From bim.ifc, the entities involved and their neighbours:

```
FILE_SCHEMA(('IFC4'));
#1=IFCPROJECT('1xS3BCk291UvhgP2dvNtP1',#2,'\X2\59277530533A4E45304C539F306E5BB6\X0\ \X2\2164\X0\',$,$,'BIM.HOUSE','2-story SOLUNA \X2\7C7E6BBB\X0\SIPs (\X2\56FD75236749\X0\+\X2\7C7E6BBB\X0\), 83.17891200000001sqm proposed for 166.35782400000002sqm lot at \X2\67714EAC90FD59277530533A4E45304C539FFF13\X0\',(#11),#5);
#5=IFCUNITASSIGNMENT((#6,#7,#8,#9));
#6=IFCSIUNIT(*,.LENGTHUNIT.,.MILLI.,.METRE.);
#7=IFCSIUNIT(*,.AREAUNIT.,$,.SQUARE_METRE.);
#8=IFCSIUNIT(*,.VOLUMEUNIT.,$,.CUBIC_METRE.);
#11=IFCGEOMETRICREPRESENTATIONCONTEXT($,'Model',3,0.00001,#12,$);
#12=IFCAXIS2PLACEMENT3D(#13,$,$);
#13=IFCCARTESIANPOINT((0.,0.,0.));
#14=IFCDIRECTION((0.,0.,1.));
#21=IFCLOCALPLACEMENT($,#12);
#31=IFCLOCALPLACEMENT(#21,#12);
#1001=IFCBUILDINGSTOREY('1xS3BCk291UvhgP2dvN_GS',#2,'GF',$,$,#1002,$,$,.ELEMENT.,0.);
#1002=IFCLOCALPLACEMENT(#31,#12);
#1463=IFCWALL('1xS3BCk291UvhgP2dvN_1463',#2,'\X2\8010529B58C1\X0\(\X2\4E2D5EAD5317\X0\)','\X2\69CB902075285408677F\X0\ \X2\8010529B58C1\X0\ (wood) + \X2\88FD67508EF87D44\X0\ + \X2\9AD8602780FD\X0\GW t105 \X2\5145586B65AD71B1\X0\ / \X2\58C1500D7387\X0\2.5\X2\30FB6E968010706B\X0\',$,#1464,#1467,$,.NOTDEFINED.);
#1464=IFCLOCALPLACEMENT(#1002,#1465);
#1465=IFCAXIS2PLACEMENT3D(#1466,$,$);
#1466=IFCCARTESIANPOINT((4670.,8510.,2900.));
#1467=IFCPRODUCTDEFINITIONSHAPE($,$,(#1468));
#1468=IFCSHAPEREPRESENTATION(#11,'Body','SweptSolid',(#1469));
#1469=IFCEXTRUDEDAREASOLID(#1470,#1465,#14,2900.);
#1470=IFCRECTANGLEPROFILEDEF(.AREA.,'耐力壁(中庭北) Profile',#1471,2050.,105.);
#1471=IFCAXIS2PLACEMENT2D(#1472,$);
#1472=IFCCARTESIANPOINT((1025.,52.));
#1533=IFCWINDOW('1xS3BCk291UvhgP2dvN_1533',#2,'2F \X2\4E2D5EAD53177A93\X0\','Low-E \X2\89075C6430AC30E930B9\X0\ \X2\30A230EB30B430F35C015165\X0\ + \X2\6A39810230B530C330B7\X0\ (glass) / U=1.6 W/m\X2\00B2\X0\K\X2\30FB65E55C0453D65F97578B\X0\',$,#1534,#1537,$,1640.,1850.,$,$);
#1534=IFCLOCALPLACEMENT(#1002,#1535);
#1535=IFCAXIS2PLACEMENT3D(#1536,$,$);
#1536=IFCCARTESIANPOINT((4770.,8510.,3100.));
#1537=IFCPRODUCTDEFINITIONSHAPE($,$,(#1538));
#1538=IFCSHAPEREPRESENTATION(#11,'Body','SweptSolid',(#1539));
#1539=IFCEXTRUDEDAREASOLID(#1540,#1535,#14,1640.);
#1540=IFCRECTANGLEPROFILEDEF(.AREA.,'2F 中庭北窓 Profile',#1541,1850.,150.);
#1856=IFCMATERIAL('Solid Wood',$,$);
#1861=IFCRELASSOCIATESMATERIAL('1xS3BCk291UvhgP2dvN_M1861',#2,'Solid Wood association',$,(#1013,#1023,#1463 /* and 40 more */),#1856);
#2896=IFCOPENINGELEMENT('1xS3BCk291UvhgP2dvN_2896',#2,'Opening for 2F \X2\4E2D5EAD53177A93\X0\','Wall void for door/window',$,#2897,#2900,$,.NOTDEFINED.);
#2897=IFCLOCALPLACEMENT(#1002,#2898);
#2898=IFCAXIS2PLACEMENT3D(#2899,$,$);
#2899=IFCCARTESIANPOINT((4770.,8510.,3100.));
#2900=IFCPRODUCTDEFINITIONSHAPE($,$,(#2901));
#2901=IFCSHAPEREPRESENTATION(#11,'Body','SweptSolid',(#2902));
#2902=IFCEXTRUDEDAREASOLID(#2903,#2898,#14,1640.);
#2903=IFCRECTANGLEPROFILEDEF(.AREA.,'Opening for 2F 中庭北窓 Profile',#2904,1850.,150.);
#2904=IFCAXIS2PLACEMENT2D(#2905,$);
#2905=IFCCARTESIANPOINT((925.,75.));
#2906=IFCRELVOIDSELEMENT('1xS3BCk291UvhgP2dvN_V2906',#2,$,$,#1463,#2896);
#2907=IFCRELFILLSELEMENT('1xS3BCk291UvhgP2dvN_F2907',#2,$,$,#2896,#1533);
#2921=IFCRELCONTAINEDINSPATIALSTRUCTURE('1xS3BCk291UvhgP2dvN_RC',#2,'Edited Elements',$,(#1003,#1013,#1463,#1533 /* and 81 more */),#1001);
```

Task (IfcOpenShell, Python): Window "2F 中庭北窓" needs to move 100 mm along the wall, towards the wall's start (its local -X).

```python
import ifcopenshell
import ifcopenshell.api.geometry
import ifcopenshell.util.placement
import ifcopenshell.util.unit

model = ifcopenshell.open("bim.ifc")
unit_scale = ifcopenshell.util.unit.calculate_unit_scale(model)

window = model.by_guid("1xS3BCk291UvhgP2dvN_1533")
opening = window.FillsVoids[0].RelatingOpeningElement
wall = opening.VoidsElements[0].RelatingBuildingElement

wall_matrix = ifcopenshell.util.placement.get_local_placement(wall.ObjectPlacement)
shift = wall_matrix[:3, 0] * -0.1 / unit_scale
before = ifcopenshell.util.placement.get_local_placement(window.ObjectPlacement)[:3, 3].copy()

# The window is not placed relative to its opening, so move both.
for product in (opening, window):
    matrix = ifcopenshell.util.placement.get_local_placement(product.ObjectPlacement)
    matrix[:3, 3] += shift
    ifcopenshell.api.geometry.edit_object_placement(model, product=product, matrix=matrix, is_si=False)

after = ifcopenshell.util.placement.get_local_placement(window.ObjectPlacement)[:3, 3]
print("window moved by", (after - before).round(3) + 0.0)

model.write("bim-out.ifc")
```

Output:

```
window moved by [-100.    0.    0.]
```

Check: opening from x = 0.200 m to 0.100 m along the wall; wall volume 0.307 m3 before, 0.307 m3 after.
